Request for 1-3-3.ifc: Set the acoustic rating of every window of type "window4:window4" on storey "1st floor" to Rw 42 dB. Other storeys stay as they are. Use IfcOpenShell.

First a look at what the model holds.

```python
import ifcopenshell
import ifcopenshell.util.element

model = ifcopenshell.open("1-3-3.ifc")
print(model.schema)
storey = next(s for s in model.by_type("IfcBuildingStorey") if s.Name == "1st floor")
windows = [e for e in ifcopenshell.util.element.get_decomposition(storey) if e.is_a("IfcWindow")]
seen = {}
for e in windows:
    element_type = ifcopenshell.util.element.get_type(e)
    key = (element_type.Name if element_type != e and element_type else None, ifcopenshell.util.element.get_pset(e, "Pset_WindowCommon", "AcousticRating"))
    seen[key] = seen.get(key, 0) + 1
for (name, value), count in sorted(seen.items(), key=str):
    print(count, "x", name, "|", value)
```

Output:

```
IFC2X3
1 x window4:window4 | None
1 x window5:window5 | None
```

```python
import ifcopenshell
import ifcopenshell.api.pset
import ifcopenshell.util.element

model = ifcopenshell.open("1-3-3.ifc")

storey = next(s for s in model.by_type("IfcBuildingStorey") if s.Name == "1st floor")
windows = [e for e in ifcopenshell.util.element.get_decomposition(storey) if e.is_a("IfcWindow")]

count = 0
for e in windows:
    element_type = ifcopenshell.util.element.get_type(e)
    if element_type in (None, e) or element_type.Name != "window4:window4":
        continue
    # add_pset returns the element's existing set when there is one.
    pset = ifcopenshell.api.pset.add_pset(model, product=e, name="Pset_WindowCommon")
    ifcopenshell.api.pset.edit_pset(model, pset=pset, properties={"AcousticRating": "Rw 42 dB"})
    count += 1

print(count, "windows updated")

model.write("1-3-3-out.ifc")
```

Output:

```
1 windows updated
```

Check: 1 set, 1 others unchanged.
